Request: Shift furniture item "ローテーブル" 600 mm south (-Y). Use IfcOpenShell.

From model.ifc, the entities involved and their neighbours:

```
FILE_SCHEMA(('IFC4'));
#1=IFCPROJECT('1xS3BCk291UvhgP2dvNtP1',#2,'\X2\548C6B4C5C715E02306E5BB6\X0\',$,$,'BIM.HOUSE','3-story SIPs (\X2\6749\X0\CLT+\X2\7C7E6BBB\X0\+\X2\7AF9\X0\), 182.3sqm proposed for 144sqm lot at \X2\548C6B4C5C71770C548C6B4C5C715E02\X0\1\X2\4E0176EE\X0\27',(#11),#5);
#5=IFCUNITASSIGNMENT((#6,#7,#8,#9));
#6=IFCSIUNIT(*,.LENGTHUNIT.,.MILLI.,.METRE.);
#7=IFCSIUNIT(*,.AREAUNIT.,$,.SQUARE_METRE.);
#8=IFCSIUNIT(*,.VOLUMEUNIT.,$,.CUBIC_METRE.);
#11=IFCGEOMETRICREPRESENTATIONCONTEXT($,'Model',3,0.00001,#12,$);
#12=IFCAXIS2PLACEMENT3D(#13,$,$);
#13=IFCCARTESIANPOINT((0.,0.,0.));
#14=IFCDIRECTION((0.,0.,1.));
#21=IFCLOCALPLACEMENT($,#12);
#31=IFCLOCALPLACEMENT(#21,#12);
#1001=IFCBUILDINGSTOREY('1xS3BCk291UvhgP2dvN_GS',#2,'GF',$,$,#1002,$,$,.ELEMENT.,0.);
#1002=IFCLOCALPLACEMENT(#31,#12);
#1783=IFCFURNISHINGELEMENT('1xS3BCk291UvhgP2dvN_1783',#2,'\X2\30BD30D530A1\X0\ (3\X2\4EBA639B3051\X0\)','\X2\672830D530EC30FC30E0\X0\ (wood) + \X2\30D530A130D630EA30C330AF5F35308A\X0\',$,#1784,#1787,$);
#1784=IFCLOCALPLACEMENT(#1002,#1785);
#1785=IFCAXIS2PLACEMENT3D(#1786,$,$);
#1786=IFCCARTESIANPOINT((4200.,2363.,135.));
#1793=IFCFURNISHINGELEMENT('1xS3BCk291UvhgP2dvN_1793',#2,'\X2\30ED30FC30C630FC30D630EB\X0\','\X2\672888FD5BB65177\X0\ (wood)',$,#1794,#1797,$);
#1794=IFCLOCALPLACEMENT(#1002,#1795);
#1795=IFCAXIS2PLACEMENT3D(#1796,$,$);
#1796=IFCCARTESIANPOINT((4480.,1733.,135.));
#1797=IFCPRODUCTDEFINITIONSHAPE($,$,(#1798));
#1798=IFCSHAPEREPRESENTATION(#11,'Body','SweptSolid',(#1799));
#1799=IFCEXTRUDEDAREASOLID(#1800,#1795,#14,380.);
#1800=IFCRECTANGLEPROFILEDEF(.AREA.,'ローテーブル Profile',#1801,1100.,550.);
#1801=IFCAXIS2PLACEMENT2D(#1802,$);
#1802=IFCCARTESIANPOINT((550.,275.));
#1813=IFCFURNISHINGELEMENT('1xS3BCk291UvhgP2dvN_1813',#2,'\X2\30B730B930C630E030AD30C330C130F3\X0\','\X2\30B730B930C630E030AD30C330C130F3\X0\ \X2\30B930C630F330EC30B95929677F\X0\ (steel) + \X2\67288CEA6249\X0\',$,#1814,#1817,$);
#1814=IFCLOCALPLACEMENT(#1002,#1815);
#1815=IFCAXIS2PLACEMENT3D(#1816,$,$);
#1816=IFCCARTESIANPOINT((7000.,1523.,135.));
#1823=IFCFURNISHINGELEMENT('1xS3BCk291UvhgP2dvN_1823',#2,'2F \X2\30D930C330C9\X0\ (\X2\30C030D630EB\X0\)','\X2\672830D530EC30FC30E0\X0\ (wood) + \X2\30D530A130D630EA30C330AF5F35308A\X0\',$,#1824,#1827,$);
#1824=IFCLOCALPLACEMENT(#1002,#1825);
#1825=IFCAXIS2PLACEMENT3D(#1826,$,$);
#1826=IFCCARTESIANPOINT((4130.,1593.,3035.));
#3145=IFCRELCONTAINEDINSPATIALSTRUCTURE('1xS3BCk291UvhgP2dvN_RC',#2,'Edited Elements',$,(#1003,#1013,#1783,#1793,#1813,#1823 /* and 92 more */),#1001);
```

```python
import ifcopenshell
import ifcopenshell.api.geometry
import ifcopenshell.util.placement
import ifcopenshell.util.unit

model = ifcopenshell.open("model.ifc")
unit_scale = ifcopenshell.util.unit.calculate_unit_scale(model)

item = model.by_guid("1xS3BCk291UvhgP2dvN_1793")
matrix = ifcopenshell.util.placement.get_local_placement(item.ObjectPlacement)
matrix[1, 3] -= 0.6 / unit_scale
ifcopenshell.api.geometry.edit_object_placement(model, product=item, matrix=matrix, is_si=False)

print(ifcopenshell.util.placement.get_local_placement(item.ObjectPlacement).round(3) + 0.0)

model.write("model_updated.ifc")
```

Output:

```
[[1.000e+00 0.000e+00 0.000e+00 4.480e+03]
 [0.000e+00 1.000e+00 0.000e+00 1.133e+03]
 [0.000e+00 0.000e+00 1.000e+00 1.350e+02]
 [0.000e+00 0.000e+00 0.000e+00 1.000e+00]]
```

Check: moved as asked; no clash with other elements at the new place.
